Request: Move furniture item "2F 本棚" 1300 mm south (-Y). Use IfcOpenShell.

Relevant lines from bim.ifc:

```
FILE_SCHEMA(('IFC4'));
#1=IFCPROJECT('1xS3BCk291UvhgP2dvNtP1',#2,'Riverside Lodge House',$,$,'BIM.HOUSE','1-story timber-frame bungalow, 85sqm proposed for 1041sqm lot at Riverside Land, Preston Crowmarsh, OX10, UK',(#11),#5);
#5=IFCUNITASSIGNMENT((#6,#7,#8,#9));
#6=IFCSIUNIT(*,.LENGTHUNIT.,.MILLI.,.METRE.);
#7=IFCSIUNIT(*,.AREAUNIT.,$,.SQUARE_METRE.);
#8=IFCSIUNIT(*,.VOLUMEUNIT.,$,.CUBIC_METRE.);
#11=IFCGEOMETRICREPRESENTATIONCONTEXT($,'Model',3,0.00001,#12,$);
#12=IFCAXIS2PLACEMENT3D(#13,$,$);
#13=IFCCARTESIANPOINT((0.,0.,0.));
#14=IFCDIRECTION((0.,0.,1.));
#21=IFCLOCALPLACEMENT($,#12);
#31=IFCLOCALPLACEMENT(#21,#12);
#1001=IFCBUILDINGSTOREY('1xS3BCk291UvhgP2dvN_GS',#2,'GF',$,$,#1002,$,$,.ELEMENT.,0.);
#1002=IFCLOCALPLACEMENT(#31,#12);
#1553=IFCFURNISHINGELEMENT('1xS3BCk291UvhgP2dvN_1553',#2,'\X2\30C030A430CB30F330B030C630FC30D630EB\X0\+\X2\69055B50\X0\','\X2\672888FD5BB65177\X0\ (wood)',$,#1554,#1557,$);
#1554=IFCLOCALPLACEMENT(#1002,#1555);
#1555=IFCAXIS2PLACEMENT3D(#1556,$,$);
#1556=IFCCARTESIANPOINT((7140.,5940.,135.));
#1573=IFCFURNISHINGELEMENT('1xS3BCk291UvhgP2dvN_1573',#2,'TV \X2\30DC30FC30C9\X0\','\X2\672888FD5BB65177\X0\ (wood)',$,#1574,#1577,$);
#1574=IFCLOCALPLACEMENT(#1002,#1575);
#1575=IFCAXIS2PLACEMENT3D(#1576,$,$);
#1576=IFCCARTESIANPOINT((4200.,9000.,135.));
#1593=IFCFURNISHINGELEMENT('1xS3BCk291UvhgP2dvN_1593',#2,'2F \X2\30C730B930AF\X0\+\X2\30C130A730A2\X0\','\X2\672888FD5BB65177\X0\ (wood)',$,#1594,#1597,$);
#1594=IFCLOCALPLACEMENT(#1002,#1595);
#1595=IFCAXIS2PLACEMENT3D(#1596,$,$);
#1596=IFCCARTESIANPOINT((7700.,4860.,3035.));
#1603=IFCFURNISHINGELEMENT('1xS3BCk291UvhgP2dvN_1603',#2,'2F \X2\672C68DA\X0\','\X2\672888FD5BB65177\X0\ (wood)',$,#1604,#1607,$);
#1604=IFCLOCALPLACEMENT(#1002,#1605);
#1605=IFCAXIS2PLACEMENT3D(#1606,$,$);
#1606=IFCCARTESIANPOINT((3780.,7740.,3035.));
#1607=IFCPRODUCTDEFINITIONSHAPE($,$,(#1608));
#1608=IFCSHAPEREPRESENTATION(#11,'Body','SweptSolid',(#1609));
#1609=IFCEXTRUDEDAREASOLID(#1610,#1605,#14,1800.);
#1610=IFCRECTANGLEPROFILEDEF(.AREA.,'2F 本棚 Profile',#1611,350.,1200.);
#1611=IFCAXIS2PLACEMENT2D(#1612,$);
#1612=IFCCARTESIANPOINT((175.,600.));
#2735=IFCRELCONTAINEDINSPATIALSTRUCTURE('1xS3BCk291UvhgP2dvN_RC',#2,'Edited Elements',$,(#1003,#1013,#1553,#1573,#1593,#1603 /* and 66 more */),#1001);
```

```python
import ifcopenshell
import ifcopenshell.api.geometry
import ifcopenshell.util.placement
import ifcopenshell.util.unit

model = ifcopenshell.open("bim.ifc")
unit_scale = ifcopenshell.util.unit.calculate_unit_scale(model)

item = model.by_guid("1xS3BCk291UvhgP2dvN_1603")
matrix = ifcopenshell.util.placement.get_local_placement(item.ObjectPlacement)
matrix[1, 3] -= 1.3 / unit_scale
ifcopenshell.api.geometry.edit_object_placement(model, product=item, matrix=matrix, is_si=False)

print(ifcopenshell.util.placement.get_local_placement(item.ObjectPlacement).round(3) + 0.0)

model.write("bim_edited.ifc")
```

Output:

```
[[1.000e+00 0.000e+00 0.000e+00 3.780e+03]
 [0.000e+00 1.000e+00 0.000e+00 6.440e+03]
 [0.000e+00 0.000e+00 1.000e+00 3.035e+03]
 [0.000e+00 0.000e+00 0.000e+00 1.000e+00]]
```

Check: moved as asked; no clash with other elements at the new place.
